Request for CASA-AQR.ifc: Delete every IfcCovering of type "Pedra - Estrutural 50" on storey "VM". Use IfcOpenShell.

First a look at what the model holds.

```python
import ifcopenshell
import ifcopenshell.util.element

model = ifcopenshell.open("CASA-AQR.ifc")
print(model.schema)
storey = next(s for s in model.by_type("IfcBuildingStorey") if s.Name == "VM")
coverings = [e for e in ifcopenshell.util.element.get_decomposition(storey) if e.is_a("IfcCovering")]
seen = {}
for e in coverings:
    element_type = ifcopenshell.util.element.get_type(e)
    name = element_type.Name if element_type not in (None, e) else None
    seen[name] = seen.get(name, 0) + 1
for name, count in sorted(seen.items(), key=str):
    print(count, "x", name)
```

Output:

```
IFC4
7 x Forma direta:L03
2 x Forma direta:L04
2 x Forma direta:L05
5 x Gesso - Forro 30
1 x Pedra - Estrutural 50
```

```python
import ifcopenshell
import ifcopenshell.api.root
import ifcopenshell.util.element

model = ifcopenshell.open("CASA-AQR.ifc")

storey = next(s for s in model.by_type("IfcBuildingStorey") if s.Name == "VM")
coverings = [e for e in ifcopenshell.util.element.get_decomposition(storey) if e.is_a("IfcCovering")]
targets = [e for e in coverings if (t := ifcopenshell.util.element.get_type(e)) not in (None, e) and t.Name == "Pedra - Estrutural 50"]

for e in targets:
    ifcopenshell.api.root.remove_product(model, product=e)
print(len(targets), "removed")

model.write("CASA-AQR_edited.ifc")
```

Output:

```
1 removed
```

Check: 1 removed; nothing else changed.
